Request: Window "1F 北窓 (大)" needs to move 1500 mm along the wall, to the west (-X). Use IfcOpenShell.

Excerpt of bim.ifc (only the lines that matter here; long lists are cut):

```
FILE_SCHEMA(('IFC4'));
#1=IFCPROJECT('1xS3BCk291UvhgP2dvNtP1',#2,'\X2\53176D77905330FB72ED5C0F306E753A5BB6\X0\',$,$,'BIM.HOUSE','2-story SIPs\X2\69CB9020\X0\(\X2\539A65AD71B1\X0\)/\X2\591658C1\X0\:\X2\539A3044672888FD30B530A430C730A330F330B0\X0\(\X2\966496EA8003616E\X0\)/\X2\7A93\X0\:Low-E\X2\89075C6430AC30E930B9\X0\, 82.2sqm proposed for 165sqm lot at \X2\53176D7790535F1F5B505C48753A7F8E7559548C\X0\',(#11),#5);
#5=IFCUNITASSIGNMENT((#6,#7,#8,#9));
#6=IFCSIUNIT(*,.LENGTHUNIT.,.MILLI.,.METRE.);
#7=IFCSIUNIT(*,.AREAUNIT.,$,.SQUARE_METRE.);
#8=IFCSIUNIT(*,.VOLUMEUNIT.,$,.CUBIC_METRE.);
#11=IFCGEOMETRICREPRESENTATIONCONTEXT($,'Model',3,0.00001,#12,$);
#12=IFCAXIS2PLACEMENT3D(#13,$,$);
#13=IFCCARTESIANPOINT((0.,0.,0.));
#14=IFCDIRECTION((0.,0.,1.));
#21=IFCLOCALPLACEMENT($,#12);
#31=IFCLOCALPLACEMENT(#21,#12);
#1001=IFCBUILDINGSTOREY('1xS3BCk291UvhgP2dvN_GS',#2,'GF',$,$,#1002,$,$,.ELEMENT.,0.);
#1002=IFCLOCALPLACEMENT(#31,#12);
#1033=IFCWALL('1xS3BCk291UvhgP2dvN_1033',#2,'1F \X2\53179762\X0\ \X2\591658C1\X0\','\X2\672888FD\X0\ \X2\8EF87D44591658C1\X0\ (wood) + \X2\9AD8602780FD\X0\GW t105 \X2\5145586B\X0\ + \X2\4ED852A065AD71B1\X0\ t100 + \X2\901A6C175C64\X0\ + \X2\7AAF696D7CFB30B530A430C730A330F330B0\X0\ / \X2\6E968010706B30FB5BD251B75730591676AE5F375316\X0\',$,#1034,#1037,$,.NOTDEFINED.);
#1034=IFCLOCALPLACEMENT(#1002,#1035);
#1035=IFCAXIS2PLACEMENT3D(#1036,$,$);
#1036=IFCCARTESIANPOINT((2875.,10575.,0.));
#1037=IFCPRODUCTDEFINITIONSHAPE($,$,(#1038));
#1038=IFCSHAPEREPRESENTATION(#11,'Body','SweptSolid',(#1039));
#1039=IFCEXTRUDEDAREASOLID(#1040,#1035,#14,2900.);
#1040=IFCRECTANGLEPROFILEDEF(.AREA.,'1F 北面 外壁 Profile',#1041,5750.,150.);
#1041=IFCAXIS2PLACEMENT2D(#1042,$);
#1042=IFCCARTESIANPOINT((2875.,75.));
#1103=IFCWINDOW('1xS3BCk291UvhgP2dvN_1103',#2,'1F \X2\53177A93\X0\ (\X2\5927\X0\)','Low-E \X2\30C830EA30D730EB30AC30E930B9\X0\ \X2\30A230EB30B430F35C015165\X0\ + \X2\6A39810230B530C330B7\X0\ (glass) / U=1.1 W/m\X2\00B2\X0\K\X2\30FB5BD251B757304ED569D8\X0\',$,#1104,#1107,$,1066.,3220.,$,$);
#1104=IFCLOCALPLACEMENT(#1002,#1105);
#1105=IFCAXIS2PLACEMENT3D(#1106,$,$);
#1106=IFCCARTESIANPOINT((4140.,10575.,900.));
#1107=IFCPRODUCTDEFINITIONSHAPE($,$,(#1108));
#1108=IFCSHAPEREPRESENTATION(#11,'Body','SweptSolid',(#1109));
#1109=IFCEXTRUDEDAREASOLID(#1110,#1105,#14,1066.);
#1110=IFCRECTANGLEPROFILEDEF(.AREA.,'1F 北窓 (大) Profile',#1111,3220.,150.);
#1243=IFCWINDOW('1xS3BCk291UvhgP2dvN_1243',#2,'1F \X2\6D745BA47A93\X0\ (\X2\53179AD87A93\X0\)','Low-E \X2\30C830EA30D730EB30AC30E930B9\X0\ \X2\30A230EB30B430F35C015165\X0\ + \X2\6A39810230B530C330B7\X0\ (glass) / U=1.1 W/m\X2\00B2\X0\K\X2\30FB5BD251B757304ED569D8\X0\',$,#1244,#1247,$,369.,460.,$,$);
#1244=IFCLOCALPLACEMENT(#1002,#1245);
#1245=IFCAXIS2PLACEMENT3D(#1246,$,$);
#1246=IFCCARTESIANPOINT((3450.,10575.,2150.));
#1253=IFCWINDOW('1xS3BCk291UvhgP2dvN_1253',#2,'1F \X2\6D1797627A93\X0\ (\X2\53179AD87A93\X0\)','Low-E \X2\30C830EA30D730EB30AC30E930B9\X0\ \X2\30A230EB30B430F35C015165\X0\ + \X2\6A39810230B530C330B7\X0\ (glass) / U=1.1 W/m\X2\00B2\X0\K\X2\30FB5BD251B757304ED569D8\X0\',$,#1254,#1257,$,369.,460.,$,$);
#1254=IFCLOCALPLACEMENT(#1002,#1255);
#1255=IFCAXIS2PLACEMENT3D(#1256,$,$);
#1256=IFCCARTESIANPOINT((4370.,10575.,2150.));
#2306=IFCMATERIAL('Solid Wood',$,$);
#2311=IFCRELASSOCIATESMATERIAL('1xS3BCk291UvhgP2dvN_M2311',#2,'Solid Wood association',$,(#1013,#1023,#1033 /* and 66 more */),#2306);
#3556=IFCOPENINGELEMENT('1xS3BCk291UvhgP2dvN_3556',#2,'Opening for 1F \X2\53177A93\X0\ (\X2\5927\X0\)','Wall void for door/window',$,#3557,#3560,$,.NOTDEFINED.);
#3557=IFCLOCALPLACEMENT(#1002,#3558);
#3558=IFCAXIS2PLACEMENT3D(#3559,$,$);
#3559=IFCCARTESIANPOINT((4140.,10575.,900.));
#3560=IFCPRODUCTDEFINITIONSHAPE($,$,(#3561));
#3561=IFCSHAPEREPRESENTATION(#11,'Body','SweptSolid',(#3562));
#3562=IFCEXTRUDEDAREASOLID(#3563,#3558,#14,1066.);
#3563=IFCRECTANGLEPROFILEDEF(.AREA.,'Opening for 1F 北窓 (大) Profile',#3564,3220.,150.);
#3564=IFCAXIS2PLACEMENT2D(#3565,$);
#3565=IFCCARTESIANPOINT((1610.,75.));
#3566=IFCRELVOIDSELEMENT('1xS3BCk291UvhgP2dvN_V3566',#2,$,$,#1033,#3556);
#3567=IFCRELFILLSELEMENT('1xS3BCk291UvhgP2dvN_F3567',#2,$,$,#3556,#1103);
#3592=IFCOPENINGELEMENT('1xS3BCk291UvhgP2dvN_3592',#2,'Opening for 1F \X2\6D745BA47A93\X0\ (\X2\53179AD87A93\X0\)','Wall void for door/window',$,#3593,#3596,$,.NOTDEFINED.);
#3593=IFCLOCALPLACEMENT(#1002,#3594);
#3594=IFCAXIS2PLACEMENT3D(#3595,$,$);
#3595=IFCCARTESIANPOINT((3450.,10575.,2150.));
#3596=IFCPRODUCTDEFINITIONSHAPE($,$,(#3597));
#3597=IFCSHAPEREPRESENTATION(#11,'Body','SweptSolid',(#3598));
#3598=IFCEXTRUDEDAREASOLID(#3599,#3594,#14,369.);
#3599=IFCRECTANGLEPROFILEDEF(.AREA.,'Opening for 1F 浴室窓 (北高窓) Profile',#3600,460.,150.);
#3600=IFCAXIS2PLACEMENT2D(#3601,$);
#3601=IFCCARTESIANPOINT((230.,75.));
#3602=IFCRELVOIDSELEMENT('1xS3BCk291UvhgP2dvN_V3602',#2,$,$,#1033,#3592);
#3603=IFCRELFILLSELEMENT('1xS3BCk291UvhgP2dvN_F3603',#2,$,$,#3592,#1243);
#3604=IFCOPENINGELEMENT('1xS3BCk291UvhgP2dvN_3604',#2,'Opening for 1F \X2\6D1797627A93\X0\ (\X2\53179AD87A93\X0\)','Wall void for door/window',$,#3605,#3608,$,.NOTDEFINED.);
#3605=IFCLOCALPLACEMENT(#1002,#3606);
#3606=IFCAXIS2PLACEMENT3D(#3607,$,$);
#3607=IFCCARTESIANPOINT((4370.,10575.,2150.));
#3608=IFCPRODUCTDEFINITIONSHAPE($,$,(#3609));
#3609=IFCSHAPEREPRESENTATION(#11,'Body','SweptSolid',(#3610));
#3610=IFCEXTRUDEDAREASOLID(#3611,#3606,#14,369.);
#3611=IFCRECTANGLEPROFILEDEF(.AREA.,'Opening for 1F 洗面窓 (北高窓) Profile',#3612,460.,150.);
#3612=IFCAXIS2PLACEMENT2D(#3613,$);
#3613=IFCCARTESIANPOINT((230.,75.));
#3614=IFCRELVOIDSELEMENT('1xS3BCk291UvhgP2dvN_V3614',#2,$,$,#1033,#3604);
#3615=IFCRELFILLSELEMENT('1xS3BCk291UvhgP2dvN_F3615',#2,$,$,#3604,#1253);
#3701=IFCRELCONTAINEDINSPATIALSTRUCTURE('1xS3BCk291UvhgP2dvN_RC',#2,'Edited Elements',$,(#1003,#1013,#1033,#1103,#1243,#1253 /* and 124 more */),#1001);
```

```python
import ifcopenshell
import ifcopenshell.api.geometry
import ifcopenshell.util.placement

model = ifcopenshell.open("bim.ifc")

window = model.by_guid("1xS3BCk291UvhgP2dvN_1103")
opening = window.FillsVoids[0].RelatingOpeningElement
wall = opening.VoidsElements[0].RelatingBuildingElement

wall_matrix = ifcopenshell.util.placement.get_local_placement(wall.ObjectPlacement)
shift = wall_matrix[:3, 0] * -1500.0
before = ifcopenshell.util.placement.get_local_placement(window.ObjectPlacement)[:3, 3].copy()

# The window is not placed relative to its opening, so move both.
for product in (opening, window):
    matrix = ifcopenshell.util.placement.get_local_placement(product.ObjectPlacement)
    matrix[:3, 3] += shift
    ifcopenshell.api.geometry.edit_object_placement(model, product=product, matrix=matrix, is_si=False)

after = ifcopenshell.util.placement.get_local_placement(window.ObjectPlacement)[:3, 3]
print("window moved by", (after - before).round(3) + 0.0)

model.write("bim_rev.ifc")
```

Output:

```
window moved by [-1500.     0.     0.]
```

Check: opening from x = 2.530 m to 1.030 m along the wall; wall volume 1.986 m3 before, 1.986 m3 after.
